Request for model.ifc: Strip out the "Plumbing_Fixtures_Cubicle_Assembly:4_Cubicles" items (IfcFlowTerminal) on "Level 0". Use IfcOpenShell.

First a look at what the model holds.

```python
import ifcopenshell
import ifcopenshell.util.element

model = ifcopenshell.open("model.ifc")
print(model.schema)
storey = next(s for s in model.by_type("IfcBuildingStorey") if s.Name == "Level 0")
terminals = [e for e in ifcopenshell.util.element.get_decomposition(storey) if e.is_a("IfcFlowTerminal")]
seen = {}
for e in terminals:
    element_type = ifcopenshell.util.element.get_type(e)
    name = element_type.Name if element_type not in (None, e) else None
    seen[name] = seen.get(name, 0) + 1
for name, count in sorted(seen.items(), key=str):
    print(count, "x", name)
```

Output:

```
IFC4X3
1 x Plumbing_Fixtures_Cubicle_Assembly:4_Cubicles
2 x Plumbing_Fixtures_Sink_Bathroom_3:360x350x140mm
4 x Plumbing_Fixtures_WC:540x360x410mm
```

```python
import ifcopenshell
import ifcopenshell.api.root
import ifcopenshell.util.element

model = ifcopenshell.open("model.ifc")

storey = next(s for s in model.by_type("IfcBuildingStorey") if s.Name == "Level 0")
terminals = [e for e in ifcopenshell.util.element.get_decomposition(storey) if e.is_a("IfcFlowTerminal")]
targets = [e for e in terminals if (t := ifcopenshell.util.element.get_type(e)) not in (None, e) and t.Name == "Plumbing_Fixtures_Cubicle_Assembly:4_Cubicles"]

for e in targets:
    ifcopenshell.api.root.remove_product(model, product=e)
print(len(targets), "removed")

model.write("model-out.ifc")
```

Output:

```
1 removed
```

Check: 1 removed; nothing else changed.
